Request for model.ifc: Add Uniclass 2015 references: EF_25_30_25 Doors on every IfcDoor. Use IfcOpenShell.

First a look at what the model holds.

```python
import ifcopenshell

model = ifcopenshell.open("model.ifc")
print(model.schema)
print("classifications:", [c.Name for c in model.by_type("IfcClassification")])
for ifc_class in ("IfcDoor", "IfcRoof", "IfcStair", "IfcWall", "IfcWindow"):
    print(ifc_class, len(model.by_type(ifc_class)))
```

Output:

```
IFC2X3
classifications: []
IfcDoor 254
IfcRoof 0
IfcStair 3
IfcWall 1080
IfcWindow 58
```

```python
import ifcopenshell
import ifcopenshell.api.classification

model = ifcopenshell.open("model.ifc")

# IFC2X3 requires Source and Edition and has no link from the project to the system.
system = model.create_entity("IfcClassification", Source="NBS", Edition="2015", Name="Uniclass 2015")

codes = {
    "IfcDoor": ("EF_25_30_25", "Doors"),
}
for ifc_class, (code, name) in codes.items():
    products = model.by_type(ifc_class)
    ifcopenshell.api.classification.add_reference(
        model, products=products, classification=system, identification=code, name=name
    )
    print(code, len(products))

model.write("model_updated.ifc")
```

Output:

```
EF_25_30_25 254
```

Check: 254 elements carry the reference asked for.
